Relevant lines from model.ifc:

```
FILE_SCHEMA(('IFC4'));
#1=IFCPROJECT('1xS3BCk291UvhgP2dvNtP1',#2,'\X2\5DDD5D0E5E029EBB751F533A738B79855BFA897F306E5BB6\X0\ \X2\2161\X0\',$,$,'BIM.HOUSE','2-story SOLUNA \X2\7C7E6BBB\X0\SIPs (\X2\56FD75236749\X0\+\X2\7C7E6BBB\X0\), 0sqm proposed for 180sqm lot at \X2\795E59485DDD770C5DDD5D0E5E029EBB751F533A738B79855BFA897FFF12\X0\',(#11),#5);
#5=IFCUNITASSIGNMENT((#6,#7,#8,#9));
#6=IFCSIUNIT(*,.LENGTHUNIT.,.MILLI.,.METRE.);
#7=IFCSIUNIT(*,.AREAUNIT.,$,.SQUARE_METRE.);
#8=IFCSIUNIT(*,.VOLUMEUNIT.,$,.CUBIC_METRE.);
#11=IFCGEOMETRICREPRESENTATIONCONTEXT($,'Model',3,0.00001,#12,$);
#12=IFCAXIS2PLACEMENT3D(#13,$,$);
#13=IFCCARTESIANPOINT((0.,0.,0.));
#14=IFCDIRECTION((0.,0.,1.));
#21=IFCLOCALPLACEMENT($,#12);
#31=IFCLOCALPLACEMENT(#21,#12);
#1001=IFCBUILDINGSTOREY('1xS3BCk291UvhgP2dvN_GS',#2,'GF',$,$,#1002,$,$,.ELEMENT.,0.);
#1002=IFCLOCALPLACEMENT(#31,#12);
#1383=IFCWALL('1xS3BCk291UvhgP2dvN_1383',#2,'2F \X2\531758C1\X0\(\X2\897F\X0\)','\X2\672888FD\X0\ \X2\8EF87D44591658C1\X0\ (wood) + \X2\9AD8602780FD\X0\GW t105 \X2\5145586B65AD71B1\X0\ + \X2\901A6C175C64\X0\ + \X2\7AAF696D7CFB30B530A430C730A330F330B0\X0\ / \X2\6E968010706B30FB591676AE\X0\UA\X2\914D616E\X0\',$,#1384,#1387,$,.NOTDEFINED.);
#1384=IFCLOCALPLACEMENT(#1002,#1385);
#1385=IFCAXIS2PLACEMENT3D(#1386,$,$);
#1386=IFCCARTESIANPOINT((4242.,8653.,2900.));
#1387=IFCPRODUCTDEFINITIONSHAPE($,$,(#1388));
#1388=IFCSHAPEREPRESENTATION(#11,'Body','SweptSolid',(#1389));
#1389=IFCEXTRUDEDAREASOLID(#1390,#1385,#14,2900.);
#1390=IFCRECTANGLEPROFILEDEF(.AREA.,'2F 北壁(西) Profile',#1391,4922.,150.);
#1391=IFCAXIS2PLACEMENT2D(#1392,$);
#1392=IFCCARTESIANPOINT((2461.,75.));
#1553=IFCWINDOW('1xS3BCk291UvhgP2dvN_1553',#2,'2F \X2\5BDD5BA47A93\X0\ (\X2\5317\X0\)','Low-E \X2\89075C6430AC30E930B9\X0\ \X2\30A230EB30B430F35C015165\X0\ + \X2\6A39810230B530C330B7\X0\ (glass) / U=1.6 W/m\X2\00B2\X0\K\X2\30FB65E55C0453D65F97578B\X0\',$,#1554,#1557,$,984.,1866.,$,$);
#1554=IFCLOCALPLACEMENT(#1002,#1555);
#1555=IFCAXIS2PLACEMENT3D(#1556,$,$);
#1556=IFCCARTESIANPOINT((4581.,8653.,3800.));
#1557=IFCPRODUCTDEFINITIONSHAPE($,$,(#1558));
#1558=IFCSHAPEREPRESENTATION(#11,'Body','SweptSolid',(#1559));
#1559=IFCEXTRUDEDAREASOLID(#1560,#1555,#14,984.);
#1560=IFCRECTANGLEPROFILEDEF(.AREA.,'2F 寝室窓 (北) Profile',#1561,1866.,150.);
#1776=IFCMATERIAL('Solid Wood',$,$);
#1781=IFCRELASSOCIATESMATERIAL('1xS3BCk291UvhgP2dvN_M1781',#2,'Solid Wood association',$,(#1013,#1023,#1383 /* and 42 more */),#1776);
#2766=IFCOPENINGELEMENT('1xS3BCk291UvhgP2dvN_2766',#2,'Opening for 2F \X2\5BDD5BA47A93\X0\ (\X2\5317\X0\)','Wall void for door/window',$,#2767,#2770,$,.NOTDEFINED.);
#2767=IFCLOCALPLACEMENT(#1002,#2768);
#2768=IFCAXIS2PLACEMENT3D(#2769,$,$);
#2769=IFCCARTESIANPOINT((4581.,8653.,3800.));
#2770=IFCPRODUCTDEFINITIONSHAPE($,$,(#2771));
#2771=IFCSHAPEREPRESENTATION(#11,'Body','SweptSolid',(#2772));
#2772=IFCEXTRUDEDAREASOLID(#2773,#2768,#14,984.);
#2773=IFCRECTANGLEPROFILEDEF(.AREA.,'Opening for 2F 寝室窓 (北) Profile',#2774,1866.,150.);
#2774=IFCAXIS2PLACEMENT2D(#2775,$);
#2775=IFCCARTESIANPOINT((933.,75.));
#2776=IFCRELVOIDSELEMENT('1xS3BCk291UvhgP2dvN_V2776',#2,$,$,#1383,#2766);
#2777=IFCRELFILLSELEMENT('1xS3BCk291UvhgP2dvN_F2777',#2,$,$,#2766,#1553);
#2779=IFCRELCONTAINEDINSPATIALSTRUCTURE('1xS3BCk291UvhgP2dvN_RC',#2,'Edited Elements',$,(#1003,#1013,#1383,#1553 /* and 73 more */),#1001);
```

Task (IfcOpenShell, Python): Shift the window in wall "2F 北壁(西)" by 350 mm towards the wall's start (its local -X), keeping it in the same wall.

```python
import ifcopenshell
import ifcopenshell.api.geometry
import ifcopenshell.util.placement

model = ifcopenshell.open("model.ifc")

window = model.by_guid("1xS3BCk291UvhgP2dvN_1553")
opening = window.FillsVoids[0].RelatingOpeningElement
wall = opening.VoidsElements[0].RelatingBuildingElement

wall_matrix = ifcopenshell.util.placement.get_local_placement(wall.ObjectPlacement)
shift = wall_matrix[:3, 0] * -350.0
before = ifcopenshell.util.placement.get_local_placement(window.ObjectPlacement)[:3, 3].copy()

# The window is not placed relative to its opening, so move both.
for product in (opening, window):
    matrix = ifcopenshell.util.placement.get_local_placement(product.ObjectPlacement)
    matrix[:3, 3] += shift
    ifcopenshell.api.geometry.edit_object_placement(model, product=product, matrix=matrix, is_si=False)

after = ifcopenshell.util.placement.get_local_placement(window.ObjectPlacement)[:3, 3]
print("window moved by", (after - before).round(3) + 0.0)

model.write("model_v2.ifc")
```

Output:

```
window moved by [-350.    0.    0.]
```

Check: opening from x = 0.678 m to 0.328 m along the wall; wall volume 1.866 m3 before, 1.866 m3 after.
